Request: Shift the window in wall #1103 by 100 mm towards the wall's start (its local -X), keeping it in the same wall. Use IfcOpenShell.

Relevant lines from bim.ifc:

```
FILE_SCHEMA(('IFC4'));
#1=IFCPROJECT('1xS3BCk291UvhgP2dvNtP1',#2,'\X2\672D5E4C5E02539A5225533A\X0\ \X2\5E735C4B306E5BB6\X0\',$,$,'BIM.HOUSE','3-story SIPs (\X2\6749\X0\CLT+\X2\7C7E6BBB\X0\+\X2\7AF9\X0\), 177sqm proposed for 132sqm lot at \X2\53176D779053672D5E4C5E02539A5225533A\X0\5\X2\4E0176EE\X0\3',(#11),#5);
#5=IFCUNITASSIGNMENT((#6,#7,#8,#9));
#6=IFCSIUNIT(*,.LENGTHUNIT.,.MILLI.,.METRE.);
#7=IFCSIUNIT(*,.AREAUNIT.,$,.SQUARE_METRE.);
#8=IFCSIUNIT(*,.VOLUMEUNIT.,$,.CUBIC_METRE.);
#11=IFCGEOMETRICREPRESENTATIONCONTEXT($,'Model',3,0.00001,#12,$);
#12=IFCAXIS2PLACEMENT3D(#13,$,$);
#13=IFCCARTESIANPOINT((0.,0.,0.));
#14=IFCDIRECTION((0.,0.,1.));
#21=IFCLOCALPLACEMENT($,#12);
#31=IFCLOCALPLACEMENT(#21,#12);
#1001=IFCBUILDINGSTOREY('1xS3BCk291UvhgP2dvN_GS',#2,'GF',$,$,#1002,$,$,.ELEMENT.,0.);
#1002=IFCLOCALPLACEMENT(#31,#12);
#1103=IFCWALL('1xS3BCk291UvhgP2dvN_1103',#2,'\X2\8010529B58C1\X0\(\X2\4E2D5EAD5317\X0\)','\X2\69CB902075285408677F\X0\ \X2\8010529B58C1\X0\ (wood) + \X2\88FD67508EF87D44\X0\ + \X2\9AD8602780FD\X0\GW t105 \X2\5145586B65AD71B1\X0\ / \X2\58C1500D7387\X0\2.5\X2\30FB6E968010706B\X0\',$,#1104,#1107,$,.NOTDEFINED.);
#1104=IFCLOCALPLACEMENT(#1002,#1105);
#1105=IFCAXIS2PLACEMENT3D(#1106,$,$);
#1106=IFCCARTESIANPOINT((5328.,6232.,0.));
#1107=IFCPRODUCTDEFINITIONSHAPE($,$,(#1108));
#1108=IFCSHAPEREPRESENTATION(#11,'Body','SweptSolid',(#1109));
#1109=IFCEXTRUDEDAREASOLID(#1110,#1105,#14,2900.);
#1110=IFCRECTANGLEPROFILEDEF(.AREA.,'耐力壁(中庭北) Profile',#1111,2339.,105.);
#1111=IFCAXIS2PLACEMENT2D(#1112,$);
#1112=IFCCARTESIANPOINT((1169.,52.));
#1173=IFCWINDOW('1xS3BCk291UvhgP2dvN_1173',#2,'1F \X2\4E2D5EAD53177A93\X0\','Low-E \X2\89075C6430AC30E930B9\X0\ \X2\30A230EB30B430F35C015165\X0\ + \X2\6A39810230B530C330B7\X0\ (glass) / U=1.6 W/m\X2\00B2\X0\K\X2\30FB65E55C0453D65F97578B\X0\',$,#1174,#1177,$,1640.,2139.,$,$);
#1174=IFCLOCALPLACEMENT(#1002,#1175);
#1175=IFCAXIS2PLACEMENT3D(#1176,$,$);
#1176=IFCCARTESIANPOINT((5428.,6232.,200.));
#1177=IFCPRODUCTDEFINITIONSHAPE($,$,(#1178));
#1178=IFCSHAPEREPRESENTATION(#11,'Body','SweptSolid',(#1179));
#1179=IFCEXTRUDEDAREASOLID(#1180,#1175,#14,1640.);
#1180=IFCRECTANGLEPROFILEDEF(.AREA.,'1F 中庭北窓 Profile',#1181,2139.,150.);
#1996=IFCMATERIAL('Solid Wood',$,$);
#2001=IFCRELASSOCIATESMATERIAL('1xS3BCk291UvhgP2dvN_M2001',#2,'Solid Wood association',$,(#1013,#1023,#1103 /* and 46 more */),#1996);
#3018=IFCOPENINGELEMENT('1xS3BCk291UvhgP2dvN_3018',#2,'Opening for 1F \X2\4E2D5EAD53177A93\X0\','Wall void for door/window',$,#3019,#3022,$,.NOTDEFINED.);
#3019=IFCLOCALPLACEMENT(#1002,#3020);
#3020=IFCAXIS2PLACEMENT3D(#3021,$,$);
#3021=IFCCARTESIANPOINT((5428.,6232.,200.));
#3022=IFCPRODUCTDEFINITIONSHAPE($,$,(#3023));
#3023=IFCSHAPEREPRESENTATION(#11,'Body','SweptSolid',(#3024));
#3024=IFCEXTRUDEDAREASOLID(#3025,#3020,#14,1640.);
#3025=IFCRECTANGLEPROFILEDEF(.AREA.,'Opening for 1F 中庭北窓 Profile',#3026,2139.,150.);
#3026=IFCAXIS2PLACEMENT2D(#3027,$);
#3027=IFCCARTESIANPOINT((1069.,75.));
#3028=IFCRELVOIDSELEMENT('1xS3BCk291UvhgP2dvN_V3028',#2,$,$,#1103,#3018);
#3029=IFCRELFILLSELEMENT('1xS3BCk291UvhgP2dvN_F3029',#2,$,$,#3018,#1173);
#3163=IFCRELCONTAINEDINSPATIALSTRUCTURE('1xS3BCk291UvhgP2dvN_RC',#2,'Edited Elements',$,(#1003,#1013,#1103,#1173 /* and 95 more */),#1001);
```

```python
import ifcopenshell
import ifcopenshell.api.geometry
import ifcopenshell.util.placement
import ifcopenshell.util.unit

model = ifcopenshell.open("bim.ifc")
unit_scale = ifcopenshell.util.unit.calculate_unit_scale(model)

window = model.by_id(1173)
opening = window.FillsVoids[0].RelatingOpeningElement
wall = opening.VoidsElements[0].RelatingBuildingElement

wall_matrix = ifcopenshell.util.placement.get_local_placement(wall.ObjectPlacement)
shift = wall_matrix[:3, 0] * -0.1 / unit_scale
before = ifcopenshell.util.placement.get_local_placement(window.ObjectPlacement)[:3, 3].copy()

# The window is not placed relative to its opening, so move both.
for product in (opening, window):
    matrix = ifcopenshell.util.placement.get_local_placement(product.ObjectPlacement)
    matrix[:3, 3] += shift
    ifcopenshell.api.geometry.edit_object_placement(model, product=product, matrix=matrix, is_si=False)

after = ifcopenshell.util.placement.get_local_placement(window.ObjectPlacement)[:3, 3]
print("window moved by", (after - before).round(3) + 0.0)

model.write("bim_updated.ifc")
```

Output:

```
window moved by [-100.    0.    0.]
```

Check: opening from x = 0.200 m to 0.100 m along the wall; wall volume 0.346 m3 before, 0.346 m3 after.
